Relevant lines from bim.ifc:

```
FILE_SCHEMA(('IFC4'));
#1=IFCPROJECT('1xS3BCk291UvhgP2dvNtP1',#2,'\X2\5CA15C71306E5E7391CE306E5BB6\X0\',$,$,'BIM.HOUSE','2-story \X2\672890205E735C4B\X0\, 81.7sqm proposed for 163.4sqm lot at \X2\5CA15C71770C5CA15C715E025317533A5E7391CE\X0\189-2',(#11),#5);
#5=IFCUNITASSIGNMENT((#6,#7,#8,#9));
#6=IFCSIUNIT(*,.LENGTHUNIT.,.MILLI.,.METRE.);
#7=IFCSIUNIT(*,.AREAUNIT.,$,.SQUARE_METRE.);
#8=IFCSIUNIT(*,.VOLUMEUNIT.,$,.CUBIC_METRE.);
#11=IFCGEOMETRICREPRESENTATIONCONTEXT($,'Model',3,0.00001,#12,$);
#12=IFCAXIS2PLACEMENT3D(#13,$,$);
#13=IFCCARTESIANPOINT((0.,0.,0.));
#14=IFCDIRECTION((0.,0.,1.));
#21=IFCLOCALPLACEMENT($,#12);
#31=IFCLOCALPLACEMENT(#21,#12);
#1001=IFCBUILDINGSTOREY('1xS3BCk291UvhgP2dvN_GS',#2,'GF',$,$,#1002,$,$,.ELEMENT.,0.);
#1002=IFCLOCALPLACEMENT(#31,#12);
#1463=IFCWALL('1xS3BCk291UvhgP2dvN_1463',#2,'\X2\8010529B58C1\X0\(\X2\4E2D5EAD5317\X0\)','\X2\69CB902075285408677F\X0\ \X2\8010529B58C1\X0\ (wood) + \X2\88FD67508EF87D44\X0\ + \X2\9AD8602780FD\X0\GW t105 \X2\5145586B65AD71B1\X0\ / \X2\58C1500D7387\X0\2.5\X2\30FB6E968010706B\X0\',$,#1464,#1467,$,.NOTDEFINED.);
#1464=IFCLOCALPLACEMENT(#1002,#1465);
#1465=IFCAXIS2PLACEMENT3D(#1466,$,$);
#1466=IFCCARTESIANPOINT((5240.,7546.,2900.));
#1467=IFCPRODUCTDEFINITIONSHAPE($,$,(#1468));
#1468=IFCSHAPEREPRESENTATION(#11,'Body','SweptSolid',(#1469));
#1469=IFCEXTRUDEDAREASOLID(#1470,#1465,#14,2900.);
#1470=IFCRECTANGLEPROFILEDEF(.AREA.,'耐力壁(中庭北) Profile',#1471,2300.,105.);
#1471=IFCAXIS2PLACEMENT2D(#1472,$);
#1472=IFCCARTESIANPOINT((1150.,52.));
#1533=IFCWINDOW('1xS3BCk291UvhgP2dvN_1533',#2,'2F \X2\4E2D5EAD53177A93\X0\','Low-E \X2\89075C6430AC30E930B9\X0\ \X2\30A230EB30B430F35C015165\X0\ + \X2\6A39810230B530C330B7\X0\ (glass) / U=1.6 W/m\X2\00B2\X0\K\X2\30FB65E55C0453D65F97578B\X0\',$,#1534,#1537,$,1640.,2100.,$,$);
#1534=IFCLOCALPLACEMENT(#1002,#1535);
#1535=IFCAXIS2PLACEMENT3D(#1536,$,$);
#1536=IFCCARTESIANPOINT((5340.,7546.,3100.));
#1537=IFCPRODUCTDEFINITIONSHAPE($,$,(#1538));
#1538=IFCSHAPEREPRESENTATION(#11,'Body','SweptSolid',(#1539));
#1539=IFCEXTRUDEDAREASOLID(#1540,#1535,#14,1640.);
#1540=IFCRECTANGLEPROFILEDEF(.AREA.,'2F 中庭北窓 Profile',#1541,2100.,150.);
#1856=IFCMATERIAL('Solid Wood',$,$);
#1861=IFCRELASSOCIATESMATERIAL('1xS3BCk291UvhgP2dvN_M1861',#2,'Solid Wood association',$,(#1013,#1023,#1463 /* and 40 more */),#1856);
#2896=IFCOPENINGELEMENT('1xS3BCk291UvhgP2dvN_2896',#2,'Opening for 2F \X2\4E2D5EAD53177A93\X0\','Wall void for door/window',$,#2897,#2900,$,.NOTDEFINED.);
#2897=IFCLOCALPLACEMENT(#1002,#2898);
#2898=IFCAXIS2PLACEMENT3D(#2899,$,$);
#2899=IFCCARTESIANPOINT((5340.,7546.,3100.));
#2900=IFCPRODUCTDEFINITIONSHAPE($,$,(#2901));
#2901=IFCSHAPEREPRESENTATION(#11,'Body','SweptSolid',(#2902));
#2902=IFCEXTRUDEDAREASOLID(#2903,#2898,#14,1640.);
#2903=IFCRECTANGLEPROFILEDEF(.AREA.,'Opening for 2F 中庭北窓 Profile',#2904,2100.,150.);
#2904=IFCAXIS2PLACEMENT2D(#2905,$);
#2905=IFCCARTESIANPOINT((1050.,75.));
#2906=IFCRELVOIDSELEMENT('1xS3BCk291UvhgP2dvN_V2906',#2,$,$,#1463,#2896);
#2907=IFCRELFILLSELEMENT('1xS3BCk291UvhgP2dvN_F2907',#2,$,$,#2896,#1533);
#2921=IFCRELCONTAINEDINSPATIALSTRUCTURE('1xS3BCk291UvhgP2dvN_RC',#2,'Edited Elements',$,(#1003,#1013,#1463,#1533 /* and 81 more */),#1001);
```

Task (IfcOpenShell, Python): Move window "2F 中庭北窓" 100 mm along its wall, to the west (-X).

```python
import ifcopenshell
import ifcopenshell.api.geometry
import ifcopenshell.util.placement
import ifcopenshell.util.unit

model = ifcopenshell.open("bim.ifc")
unit_scale = ifcopenshell.util.unit.calculate_unit_scale(model)

window = model.by_guid("1xS3BCk291UvhgP2dvN_1533")
opening = window.FillsVoids[0].RelatingOpeningElement
wall = opening.VoidsElements[0].RelatingBuildingElement

wall_matrix = ifcopenshell.util.placement.get_local_placement(wall.ObjectPlacement)
shift = wall_matrix[:3, 0] * -0.1 / unit_scale
before = ifcopenshell.util.placement.get_local_placement(window.ObjectPlacement)[:3, 3].copy()

# The window is not placed relative to its opening, so move both.
for product in (opening, window):
    matrix = ifcopenshell.util.placement.get_local_placement(product.ObjectPlacement)
    matrix[:3, 3] += shift
    ifcopenshell.api.geometry.edit_object_placement(model, product=product, matrix=matrix, is_si=False)

after = ifcopenshell.util.placement.get_local_placement(window.ObjectPlacement)[:3, 3]
print("window moved by", (after - before).round(3) + 0.0)

model.write("bim_edited.ifc")
```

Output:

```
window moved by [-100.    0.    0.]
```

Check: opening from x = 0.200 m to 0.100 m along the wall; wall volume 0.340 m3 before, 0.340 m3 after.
